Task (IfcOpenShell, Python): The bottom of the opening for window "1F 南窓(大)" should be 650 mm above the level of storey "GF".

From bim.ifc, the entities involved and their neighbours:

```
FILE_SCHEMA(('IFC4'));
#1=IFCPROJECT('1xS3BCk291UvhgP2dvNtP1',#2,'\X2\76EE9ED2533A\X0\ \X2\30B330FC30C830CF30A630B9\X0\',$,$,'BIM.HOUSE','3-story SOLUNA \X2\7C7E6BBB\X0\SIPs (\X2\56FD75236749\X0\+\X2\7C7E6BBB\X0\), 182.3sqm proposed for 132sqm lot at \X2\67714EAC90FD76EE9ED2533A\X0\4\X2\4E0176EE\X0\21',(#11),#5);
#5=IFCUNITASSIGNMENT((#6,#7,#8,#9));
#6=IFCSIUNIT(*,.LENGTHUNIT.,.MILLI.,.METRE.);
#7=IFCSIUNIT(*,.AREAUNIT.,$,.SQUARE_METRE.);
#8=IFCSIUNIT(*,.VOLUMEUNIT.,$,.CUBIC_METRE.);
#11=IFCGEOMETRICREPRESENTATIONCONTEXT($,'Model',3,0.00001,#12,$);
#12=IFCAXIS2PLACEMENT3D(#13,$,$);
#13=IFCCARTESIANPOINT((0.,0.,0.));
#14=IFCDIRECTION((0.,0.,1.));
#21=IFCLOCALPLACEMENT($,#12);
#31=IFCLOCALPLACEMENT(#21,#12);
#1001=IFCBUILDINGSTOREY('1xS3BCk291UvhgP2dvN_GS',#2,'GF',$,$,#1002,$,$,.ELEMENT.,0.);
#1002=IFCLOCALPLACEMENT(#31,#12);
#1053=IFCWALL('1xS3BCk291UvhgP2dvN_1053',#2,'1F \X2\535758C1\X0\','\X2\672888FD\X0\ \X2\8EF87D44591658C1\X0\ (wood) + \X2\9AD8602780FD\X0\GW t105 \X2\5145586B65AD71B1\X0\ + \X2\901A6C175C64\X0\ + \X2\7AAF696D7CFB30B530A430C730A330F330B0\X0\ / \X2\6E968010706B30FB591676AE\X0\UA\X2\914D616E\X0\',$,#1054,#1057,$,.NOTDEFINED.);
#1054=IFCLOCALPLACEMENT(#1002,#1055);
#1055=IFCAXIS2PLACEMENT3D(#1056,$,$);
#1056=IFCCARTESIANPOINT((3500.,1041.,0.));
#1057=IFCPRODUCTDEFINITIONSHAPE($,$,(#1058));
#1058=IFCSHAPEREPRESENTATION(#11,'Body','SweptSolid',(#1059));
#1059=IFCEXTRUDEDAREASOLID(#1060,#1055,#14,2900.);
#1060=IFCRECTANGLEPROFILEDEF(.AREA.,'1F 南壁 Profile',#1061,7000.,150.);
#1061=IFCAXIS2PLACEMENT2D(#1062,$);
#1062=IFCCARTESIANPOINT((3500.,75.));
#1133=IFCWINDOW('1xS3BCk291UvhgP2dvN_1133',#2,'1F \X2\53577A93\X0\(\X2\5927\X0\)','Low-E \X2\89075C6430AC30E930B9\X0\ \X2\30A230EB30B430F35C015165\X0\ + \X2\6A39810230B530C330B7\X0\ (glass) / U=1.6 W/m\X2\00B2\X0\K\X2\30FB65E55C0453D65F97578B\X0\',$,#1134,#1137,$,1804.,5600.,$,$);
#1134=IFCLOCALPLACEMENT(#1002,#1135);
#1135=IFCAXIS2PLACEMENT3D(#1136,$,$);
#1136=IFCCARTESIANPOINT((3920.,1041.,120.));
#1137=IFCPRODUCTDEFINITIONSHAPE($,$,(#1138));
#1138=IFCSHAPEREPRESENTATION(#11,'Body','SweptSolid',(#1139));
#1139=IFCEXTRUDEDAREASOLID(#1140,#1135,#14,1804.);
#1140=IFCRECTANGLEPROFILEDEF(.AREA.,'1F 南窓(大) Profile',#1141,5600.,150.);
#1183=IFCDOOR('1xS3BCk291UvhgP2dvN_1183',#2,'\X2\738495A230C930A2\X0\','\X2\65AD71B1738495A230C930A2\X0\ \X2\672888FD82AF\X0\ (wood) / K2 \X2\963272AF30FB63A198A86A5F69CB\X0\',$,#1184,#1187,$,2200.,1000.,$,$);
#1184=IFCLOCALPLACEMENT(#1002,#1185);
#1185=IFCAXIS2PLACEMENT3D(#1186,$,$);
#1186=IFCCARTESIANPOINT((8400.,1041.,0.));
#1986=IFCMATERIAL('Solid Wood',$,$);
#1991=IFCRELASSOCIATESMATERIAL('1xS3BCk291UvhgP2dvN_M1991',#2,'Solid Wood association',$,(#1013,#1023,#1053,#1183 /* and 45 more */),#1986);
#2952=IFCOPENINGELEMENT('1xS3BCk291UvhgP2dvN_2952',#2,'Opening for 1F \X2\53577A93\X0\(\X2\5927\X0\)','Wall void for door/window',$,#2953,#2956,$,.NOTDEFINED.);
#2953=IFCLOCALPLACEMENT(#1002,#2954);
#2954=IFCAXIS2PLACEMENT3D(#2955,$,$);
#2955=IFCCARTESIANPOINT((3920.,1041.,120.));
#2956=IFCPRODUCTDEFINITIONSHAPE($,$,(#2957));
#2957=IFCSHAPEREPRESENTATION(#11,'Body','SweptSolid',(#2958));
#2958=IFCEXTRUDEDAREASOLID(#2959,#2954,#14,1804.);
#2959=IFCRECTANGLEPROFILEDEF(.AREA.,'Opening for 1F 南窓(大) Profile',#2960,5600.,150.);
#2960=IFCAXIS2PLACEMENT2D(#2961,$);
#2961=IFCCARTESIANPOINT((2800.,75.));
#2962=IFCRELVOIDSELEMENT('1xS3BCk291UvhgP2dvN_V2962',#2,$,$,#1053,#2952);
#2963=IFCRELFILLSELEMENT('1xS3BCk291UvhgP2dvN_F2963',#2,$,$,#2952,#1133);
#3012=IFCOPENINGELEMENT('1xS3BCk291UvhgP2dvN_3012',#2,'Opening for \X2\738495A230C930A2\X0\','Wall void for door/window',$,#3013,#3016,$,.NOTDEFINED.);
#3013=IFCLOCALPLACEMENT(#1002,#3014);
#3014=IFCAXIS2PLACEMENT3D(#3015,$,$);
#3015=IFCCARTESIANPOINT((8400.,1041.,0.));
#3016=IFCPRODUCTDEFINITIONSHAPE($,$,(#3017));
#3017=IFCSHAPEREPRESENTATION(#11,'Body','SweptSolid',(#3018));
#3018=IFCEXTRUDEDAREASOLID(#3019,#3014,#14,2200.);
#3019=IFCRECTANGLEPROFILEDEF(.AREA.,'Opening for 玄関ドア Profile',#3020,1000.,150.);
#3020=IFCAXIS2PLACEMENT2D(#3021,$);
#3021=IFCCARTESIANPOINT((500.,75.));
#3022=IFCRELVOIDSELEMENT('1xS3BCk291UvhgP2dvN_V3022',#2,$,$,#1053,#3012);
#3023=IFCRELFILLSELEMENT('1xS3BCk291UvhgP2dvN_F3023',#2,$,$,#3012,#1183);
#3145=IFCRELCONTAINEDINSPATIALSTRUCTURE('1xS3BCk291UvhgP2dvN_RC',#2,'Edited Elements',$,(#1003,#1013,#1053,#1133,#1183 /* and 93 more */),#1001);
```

```python
import numpy as np
import ifcopenshell
import ifcopenshell.api.geometry
import ifcopenshell.geom
import ifcopenshell.util.element
import ifcopenshell.util.placement
import ifcopenshell.util.shape
import ifcopenshell.util.unit

model = ifcopenshell.open("bim.ifc")
unit_scale = ifcopenshell.util.unit.calculate_unit_scale(model)

window = model.by_guid("1xS3BCk291UvhgP2dvN_1133")
opening = window.FillsVoids[0].RelatingOpeningElement
storey = ifcopenshell.util.element.get_container(window, ifc_class="IfcBuildingStorey")
level = ifcopenshell.util.placement.get_local_placement(storey.ObjectPlacement)[2, 3]

# The opening's origin need not be at the sill, so measure its lowest point.
shape = ifcopenshell.geom.create_shape(ifcopenshell.geom.settings(), opening)
bottom = ifcopenshell.util.shape.get_shape_bottom_elevation(shape, shape.geometry) / unit_scale
dz = level + 0.65 / unit_scale - bottom

shift = np.array([0.0, 0.0, dz])
# The window is not placed relative to its opening, so move both.
for product in (opening, window):
    matrix = ifcopenshell.util.placement.get_local_placement(product.ObjectPlacement)
    matrix[:3, 3] += shift
    ifcopenshell.api.geometry.edit_object_placement(model, product=product, matrix=matrix, is_si=False)

print(f"moved by {dz * unit_scale:+.3f} m")

model.write("bim_edited.ifc")
```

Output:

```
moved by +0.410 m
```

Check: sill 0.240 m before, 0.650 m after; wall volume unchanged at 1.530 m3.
